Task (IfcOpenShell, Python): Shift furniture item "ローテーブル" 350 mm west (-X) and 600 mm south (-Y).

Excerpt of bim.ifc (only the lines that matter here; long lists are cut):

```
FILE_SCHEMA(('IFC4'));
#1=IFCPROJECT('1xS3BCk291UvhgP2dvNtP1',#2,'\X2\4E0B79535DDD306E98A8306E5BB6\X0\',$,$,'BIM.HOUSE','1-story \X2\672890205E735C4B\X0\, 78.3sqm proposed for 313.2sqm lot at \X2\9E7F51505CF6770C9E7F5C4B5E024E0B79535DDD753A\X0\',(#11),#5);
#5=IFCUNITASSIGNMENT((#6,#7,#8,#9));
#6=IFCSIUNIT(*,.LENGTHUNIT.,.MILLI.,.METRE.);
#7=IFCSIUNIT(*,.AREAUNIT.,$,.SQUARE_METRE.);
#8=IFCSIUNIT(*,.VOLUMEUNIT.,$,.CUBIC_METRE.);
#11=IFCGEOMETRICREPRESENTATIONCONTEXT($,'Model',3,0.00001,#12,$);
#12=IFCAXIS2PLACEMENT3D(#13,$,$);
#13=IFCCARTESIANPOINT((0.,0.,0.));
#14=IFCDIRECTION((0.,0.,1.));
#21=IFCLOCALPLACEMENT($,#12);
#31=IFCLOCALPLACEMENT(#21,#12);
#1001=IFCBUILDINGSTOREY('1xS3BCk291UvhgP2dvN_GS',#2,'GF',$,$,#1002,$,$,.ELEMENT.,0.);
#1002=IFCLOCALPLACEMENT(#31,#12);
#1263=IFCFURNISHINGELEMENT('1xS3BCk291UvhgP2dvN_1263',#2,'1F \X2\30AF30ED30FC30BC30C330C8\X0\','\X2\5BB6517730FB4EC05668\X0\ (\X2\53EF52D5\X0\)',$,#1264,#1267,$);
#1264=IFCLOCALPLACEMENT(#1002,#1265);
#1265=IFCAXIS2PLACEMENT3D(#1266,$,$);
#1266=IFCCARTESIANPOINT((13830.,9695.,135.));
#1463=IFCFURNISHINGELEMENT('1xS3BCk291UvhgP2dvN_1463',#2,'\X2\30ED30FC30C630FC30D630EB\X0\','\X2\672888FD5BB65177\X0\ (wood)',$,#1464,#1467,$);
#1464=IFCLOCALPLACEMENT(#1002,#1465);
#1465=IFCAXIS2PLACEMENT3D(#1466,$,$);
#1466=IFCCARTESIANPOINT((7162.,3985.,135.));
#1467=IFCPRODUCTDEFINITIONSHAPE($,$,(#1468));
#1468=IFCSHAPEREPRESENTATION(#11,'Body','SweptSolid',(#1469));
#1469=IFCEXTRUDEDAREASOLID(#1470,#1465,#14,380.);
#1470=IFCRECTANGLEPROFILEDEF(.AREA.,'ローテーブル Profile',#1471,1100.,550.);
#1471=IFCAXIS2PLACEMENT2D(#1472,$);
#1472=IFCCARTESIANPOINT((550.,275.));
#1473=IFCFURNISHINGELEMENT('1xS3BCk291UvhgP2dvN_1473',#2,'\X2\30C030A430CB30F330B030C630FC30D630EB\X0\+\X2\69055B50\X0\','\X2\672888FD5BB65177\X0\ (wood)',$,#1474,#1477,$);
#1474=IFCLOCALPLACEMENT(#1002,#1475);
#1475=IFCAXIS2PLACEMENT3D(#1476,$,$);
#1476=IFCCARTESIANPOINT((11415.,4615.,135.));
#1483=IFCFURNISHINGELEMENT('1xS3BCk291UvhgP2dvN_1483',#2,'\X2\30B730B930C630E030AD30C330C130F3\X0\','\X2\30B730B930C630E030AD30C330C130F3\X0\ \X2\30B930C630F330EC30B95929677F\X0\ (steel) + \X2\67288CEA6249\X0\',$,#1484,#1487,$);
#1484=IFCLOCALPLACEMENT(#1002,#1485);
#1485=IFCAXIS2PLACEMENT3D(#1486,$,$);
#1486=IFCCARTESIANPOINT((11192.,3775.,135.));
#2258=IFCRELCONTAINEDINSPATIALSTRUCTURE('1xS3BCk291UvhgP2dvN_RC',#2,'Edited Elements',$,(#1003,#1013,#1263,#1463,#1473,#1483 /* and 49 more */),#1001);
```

```python
import ifcopenshell
import ifcopenshell.api.geometry
import ifcopenshell.util.placement

model = ifcopenshell.open("bim.ifc")

item = model.by_id(1463)
matrix = ifcopenshell.util.placement.get_local_placement(item.ObjectPlacement)
matrix[0, 3] -= 350.0
matrix[1, 3] -= 600.0
ifcopenshell.api.geometry.edit_object_placement(model, product=item, matrix=matrix, is_si=False)

print(ifcopenshell.util.placement.get_local_placement(item.ObjectPlacement).round(3) + 0.0)

model.write("bim_rev.ifc")
```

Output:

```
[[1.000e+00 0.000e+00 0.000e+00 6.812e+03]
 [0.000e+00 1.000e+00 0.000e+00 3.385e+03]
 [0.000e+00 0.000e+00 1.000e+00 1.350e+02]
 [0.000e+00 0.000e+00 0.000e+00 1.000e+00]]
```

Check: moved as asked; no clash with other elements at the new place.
